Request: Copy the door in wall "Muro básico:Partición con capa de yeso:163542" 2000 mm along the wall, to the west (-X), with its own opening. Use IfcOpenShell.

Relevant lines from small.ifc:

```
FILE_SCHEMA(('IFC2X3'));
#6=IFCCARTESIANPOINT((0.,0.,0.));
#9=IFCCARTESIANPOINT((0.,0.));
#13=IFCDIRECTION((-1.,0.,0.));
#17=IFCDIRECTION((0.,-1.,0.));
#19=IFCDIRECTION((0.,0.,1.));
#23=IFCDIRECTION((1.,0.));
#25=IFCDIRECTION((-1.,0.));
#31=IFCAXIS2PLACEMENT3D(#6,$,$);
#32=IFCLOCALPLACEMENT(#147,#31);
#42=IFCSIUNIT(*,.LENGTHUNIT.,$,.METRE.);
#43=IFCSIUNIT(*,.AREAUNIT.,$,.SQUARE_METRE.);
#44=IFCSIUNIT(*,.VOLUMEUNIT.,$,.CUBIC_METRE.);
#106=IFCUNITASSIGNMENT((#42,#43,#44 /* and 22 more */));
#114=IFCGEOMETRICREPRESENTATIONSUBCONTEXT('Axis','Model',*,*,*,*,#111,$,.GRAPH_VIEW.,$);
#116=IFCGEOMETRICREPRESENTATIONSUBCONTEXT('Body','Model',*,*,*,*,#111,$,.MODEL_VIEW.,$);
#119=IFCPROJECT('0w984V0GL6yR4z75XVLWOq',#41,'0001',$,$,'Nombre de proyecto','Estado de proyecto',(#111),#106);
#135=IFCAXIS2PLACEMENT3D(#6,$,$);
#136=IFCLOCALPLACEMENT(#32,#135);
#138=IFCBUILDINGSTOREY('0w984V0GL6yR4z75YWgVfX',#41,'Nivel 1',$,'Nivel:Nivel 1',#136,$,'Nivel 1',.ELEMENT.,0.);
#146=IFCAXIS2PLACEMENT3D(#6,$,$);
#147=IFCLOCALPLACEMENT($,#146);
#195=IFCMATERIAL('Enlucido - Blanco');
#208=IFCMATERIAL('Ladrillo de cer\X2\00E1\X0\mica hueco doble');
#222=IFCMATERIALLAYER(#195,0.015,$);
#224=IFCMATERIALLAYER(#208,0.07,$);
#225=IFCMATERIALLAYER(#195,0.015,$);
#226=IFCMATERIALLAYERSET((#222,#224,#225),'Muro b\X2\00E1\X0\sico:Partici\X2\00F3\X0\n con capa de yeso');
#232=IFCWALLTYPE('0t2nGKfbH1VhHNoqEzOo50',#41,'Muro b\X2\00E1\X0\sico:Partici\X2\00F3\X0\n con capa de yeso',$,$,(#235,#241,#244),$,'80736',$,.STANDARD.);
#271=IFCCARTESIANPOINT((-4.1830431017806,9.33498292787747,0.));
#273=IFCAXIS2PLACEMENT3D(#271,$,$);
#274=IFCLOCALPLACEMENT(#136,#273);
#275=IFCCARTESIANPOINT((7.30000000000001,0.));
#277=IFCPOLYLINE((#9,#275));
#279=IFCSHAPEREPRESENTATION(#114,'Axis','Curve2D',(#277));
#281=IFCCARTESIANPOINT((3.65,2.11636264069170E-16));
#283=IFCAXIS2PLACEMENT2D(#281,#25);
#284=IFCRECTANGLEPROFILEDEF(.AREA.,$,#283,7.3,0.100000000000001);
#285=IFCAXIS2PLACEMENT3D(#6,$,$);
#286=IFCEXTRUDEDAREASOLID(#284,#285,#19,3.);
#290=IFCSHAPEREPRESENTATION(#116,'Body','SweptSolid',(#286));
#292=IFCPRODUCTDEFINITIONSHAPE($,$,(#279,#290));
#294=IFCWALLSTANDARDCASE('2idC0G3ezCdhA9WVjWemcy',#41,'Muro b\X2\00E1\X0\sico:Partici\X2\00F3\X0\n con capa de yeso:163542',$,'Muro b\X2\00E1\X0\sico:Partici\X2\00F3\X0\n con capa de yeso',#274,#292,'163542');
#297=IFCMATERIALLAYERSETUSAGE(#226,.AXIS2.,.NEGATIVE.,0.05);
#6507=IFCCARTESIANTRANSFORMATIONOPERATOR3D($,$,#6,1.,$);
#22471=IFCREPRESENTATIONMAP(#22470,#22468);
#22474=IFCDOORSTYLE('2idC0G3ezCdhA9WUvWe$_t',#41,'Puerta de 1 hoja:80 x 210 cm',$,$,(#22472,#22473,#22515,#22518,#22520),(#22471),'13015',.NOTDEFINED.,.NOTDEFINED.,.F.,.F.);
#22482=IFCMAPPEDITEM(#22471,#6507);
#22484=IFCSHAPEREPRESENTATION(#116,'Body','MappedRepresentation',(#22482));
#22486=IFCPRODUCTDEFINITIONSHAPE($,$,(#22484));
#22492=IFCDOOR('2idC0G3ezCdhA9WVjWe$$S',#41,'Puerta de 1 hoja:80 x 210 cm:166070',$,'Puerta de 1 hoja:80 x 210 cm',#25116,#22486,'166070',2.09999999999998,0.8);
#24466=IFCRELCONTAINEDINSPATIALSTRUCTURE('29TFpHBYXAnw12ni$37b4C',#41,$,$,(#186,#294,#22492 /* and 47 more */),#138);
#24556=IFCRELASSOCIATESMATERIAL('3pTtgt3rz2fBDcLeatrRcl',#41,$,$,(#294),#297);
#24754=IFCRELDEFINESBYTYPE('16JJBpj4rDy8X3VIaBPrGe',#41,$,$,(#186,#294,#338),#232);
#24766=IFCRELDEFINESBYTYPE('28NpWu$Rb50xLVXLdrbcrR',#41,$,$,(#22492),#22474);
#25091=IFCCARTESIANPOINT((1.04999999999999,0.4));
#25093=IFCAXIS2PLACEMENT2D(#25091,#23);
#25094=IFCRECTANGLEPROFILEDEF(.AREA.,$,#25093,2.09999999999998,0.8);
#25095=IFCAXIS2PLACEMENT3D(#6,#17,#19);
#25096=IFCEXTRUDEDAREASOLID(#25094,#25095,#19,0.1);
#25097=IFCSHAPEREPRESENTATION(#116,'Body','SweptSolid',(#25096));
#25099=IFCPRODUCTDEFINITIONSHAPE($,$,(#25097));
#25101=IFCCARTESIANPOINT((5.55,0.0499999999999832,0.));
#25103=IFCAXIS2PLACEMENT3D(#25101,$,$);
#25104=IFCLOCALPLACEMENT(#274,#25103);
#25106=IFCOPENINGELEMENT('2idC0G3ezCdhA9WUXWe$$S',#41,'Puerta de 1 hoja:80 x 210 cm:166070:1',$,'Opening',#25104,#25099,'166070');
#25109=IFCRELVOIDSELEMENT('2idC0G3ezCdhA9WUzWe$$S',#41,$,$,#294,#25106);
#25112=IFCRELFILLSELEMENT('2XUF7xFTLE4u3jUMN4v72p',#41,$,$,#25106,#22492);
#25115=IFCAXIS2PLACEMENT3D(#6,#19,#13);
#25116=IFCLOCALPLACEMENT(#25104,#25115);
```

```python
import ifcopenshell
import ifcopenshell.api.feature
import ifcopenshell.api.geometry
import ifcopenshell.api.root
import ifcopenshell.geom
import ifcopenshell.util.element
import ifcopenshell.util.placement
import ifcopenshell.util.shape

model = ifcopenshell.open("small.ifc")
settings = ifcopenshell.geom.settings()


def volume(element):
    """Net volume in cubic metres, openings subtracted."""
    shape = ifcopenshell.geom.create_shape(settings, element)
    return ifcopenshell.util.shape.get_volume(shape.geometry)


def reuse_history(source, copy):
    """copy_class also copies each property set's owner history, people and application; keep the originals."""
    for rel in copy.IsDefinedBy:
        if rel.is_a("IfcRelDefinesByProperties") and (history := rel.RelatingPropertyDefinition.OwnerHistory):
            rel.RelatingPropertyDefinition.OwnerHistory = source.OwnerHistory
            ifcopenshell.util.element.remove_deep2(model, history)


door = model.by_guid("2idC0G3ezCdhA9WVjWe$$S")
opening = door.FillsVoids[0].RelatingOpeningElement
wall = opening.VoidsElements[0].RelatingBuildingElement
before = volume(wall)
shift = ifcopenshell.util.placement.get_local_placement(wall.ObjectPlacement)[:3, 0] * -2.0

# copy_class copies the void relationship, type, container and properties, but no geometry.
new_opening = ifcopenshell.api.root.copy_class(model, product=opening)
new_opening.Representation = ifcopenshell.util.element.copy_deep(
    model, opening.Representation, exclude=["IfcGeometricRepresentationContext", "IfcRepresentationMap"]
)
new_opening.Name = "Puerta de 1 hoja:80 x 210 cm"
new_opening.Tag = None
new_door = ifcopenshell.api.root.copy_class(model, product=door)
new_door.Representation = ifcopenshell.util.element.copy_deep(
    model, door.Representation, exclude=["IfcGeometricRepresentationContext", "IfcRepresentationMap"]
)
new_door.Name = "Puerta de 1 hoja:80 x 210 cm"
new_door.Tag = None
reuse_history(door, new_door)
fills = ifcopenshell.api.feature.add_filling(model, opening=new_opening, element=new_door)
fills.OwnerHistory = new_door.OwnerHistory  # required in IFC2X3

for old, new in ((opening, new_opening), (door, new_door)):
    matrix = ifcopenshell.util.placement.get_local_placement(old.ObjectPlacement)
    matrix[:3, 3] += shift
    ifcopenshell.api.geometry.edit_object_placement(model, product=new, matrix=matrix, is_si=False)

after = volume(wall)

print(f"wall volume {before:.3f} -> {after:.3f} m3")

model.write("small_rev.ifc")
```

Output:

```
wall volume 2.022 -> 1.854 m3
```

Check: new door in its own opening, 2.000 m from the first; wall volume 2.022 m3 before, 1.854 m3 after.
